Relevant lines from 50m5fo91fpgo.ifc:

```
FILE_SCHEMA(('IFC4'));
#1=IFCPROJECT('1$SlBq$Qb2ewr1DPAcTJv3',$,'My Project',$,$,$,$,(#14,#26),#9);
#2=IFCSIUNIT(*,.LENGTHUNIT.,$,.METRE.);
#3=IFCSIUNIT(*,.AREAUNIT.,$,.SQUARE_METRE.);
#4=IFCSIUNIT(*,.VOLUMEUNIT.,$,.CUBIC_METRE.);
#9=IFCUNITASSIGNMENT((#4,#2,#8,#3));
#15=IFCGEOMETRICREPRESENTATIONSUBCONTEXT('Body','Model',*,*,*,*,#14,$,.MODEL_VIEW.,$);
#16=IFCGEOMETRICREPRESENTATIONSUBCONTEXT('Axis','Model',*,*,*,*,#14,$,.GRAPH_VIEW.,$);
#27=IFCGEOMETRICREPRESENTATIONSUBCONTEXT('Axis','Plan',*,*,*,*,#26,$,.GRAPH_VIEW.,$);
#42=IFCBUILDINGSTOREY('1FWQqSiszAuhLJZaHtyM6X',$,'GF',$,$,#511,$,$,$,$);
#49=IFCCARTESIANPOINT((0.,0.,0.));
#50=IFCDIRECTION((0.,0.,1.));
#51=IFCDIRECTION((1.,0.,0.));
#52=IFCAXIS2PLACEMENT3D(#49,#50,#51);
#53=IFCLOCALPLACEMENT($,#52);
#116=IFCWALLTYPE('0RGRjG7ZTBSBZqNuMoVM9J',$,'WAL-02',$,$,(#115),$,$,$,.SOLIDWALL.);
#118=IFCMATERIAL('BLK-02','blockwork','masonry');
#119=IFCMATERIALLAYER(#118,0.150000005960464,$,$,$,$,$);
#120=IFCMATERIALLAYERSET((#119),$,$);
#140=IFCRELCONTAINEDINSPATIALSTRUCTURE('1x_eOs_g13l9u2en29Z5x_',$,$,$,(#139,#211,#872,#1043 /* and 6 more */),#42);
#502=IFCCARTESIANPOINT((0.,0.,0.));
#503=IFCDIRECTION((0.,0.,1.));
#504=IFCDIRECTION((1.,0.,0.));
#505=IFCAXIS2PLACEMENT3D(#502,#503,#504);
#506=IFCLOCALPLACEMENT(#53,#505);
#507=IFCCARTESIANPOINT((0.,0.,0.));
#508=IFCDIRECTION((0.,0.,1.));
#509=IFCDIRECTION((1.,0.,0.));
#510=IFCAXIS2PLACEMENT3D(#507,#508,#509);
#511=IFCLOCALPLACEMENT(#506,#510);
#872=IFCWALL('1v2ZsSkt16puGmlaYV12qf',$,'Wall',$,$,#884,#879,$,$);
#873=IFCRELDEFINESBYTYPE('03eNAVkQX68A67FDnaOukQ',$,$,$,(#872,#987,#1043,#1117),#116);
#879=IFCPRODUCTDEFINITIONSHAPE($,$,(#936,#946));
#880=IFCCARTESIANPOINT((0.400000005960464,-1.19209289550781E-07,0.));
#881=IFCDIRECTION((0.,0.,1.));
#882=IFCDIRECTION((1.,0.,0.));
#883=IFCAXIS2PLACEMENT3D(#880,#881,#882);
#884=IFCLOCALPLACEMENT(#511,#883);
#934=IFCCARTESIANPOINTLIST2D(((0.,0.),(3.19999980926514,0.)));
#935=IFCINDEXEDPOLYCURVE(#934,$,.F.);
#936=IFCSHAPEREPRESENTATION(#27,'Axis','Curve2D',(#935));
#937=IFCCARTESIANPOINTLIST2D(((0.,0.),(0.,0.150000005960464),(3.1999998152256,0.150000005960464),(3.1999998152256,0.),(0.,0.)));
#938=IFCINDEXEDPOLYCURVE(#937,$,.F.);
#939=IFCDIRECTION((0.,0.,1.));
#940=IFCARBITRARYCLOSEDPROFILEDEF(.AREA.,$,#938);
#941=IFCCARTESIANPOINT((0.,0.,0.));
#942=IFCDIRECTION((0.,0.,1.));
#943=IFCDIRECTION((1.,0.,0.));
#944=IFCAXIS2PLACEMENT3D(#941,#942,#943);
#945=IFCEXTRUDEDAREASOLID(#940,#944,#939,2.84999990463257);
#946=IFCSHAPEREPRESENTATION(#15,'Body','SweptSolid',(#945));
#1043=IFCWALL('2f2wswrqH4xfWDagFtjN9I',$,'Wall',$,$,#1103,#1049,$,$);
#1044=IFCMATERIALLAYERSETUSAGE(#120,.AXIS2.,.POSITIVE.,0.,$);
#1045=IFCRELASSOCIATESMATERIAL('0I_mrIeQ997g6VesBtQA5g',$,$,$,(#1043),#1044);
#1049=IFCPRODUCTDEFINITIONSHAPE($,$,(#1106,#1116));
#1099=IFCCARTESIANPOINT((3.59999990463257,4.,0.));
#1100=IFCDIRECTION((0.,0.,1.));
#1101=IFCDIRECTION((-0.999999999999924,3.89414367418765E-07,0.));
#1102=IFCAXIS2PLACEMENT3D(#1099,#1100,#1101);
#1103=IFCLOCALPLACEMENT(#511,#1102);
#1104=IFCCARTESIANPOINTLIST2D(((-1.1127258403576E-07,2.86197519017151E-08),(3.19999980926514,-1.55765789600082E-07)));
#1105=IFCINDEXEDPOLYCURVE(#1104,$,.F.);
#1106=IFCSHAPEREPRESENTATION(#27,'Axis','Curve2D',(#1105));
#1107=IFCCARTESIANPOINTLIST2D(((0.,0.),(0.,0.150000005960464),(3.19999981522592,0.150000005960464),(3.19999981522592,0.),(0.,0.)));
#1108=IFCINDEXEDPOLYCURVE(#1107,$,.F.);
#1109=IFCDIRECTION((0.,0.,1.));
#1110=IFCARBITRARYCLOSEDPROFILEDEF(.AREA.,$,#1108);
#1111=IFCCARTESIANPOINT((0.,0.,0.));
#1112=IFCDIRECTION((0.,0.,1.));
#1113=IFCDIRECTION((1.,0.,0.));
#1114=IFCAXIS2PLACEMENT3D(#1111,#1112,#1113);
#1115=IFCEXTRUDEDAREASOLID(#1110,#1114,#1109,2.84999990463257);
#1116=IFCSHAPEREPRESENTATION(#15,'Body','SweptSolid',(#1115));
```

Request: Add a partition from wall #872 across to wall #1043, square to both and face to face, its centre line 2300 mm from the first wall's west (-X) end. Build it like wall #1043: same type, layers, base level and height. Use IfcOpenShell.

```python
import numpy as np
import ifcopenshell
import ifcopenshell.api.geometry
import ifcopenshell.api.material
import ifcopenshell.api.pset
import ifcopenshell.api.root
import ifcopenshell.api.spatial
import ifcopenshell.api.type
import ifcopenshell.geom
import ifcopenshell.util.element
import ifcopenshell.util.placement
import ifcopenshell.util.representation
import ifcopenshell.util.shape
import ifcopenshell.util.unit

model = ifcopenshell.open("50m5fo91fpgo.ifc")
unit_scale = ifcopenshell.util.unit.calculate_unit_scale(model)
settings = ifcopenshell.geom.settings()
settings.set("use-world-coords", True)

start_wall = model.by_guid("1v2ZsSkt16puGmlaYV12qf")
end_wall = model.by_id(1043)
like = model.by_id(1043)
matrix = ifcopenshell.util.placement.get_local_placement(start_wall.ObjectPlacement)
matrix[:3, 3] *= unit_scale


def extent(element):
    """Bounding box in the first wall's axes, in metres."""
    shape = ifcopenshell.geom.create_shape(settings, element)
    points = (ifcopenshell.util.shape.get_vertices(shape.geometry) - matrix[:3, 3]) @ matrix[:3, :3]
    return points.min(axis=0), points.max(axis=0)


y_start = extent(start_wall)[1][1]
y_end = extent(end_wall)[0][1]
like_min, like_max = extent(like)
length, height = float(abs(y_end - y_start)), float(like_max[2] - like_min[2])
layer_set = ifcopenshell.util.element.get_material(like, should_skip_usage=True)
thickness = sum(layer.LayerThickness for layer in layer_set.MaterialLayers) * unit_scale

wall = ifcopenshell.api.root.create_entity(model, ifc_class="IfcWall", name="New partition")
storey = ifcopenshell.util.element.get_container(like)
ifcopenshell.api.spatial.assign_container(model, products=[wall], relating_structure=storey)
ifcopenshell.api.type.assign_type(
    model, related_objects=[wall], relating_type=ifcopenshell.util.element.get_type(like), should_map_representations=False
)
rel = ifcopenshell.api.material.assign_material(
    model, products=[wall], type="IfcMaterialLayerSetUsage", material=layer_set
)
rel.RelatingMaterial.OffsetFromReferenceLine = -thickness / 2 / unit_scale
pset = ifcopenshell.api.pset.add_pset(model, product=wall, name="Pset_WallCommon")
ifcopenshell.api.pset.edit_pset(model, pset=pset, properties={"IsExternal": False, "LoadBearing": False})

# The axis runs down the middle of the wall.
axis = ifcopenshell.api.geometry.add_axis_representation(
    model, context=ifcopenshell.util.representation.get_context(model, "Model", "Axis"), axis=[(0.0, 0.0), (length, 0.0)]
)
body = ifcopenshell.api.geometry.add_wall_representation(
    model,
    context=ifcopenshell.util.representation.get_context(model, "Model", "Body", "MODEL_VIEW"),
    length=length,
    height=height,
    thickness=thickness,
    offset=-thickness / 2,
)
for representation in (axis, body):
    ifcopenshell.api.geometry.assign_representation(model, product=wall, representation=representation)

placement = matrix @ ifcopenshell.util.placement.rotation(90, "Z")
placement[:, 3] = matrix @ np.array([extent(start_wall)[0][0] + 2.3, y_start, like_min[2], 1.0])
ifcopenshell.api.geometry.edit_object_placement(model, product=wall, matrix=placement)

print(f"partition {length:.3f} m long, {height:.3f} m high, {thickness:.3f} m thick")

model.write("50m5fo91fpgo_edited.ifc")
```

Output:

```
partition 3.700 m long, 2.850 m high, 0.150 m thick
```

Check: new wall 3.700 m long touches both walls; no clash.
